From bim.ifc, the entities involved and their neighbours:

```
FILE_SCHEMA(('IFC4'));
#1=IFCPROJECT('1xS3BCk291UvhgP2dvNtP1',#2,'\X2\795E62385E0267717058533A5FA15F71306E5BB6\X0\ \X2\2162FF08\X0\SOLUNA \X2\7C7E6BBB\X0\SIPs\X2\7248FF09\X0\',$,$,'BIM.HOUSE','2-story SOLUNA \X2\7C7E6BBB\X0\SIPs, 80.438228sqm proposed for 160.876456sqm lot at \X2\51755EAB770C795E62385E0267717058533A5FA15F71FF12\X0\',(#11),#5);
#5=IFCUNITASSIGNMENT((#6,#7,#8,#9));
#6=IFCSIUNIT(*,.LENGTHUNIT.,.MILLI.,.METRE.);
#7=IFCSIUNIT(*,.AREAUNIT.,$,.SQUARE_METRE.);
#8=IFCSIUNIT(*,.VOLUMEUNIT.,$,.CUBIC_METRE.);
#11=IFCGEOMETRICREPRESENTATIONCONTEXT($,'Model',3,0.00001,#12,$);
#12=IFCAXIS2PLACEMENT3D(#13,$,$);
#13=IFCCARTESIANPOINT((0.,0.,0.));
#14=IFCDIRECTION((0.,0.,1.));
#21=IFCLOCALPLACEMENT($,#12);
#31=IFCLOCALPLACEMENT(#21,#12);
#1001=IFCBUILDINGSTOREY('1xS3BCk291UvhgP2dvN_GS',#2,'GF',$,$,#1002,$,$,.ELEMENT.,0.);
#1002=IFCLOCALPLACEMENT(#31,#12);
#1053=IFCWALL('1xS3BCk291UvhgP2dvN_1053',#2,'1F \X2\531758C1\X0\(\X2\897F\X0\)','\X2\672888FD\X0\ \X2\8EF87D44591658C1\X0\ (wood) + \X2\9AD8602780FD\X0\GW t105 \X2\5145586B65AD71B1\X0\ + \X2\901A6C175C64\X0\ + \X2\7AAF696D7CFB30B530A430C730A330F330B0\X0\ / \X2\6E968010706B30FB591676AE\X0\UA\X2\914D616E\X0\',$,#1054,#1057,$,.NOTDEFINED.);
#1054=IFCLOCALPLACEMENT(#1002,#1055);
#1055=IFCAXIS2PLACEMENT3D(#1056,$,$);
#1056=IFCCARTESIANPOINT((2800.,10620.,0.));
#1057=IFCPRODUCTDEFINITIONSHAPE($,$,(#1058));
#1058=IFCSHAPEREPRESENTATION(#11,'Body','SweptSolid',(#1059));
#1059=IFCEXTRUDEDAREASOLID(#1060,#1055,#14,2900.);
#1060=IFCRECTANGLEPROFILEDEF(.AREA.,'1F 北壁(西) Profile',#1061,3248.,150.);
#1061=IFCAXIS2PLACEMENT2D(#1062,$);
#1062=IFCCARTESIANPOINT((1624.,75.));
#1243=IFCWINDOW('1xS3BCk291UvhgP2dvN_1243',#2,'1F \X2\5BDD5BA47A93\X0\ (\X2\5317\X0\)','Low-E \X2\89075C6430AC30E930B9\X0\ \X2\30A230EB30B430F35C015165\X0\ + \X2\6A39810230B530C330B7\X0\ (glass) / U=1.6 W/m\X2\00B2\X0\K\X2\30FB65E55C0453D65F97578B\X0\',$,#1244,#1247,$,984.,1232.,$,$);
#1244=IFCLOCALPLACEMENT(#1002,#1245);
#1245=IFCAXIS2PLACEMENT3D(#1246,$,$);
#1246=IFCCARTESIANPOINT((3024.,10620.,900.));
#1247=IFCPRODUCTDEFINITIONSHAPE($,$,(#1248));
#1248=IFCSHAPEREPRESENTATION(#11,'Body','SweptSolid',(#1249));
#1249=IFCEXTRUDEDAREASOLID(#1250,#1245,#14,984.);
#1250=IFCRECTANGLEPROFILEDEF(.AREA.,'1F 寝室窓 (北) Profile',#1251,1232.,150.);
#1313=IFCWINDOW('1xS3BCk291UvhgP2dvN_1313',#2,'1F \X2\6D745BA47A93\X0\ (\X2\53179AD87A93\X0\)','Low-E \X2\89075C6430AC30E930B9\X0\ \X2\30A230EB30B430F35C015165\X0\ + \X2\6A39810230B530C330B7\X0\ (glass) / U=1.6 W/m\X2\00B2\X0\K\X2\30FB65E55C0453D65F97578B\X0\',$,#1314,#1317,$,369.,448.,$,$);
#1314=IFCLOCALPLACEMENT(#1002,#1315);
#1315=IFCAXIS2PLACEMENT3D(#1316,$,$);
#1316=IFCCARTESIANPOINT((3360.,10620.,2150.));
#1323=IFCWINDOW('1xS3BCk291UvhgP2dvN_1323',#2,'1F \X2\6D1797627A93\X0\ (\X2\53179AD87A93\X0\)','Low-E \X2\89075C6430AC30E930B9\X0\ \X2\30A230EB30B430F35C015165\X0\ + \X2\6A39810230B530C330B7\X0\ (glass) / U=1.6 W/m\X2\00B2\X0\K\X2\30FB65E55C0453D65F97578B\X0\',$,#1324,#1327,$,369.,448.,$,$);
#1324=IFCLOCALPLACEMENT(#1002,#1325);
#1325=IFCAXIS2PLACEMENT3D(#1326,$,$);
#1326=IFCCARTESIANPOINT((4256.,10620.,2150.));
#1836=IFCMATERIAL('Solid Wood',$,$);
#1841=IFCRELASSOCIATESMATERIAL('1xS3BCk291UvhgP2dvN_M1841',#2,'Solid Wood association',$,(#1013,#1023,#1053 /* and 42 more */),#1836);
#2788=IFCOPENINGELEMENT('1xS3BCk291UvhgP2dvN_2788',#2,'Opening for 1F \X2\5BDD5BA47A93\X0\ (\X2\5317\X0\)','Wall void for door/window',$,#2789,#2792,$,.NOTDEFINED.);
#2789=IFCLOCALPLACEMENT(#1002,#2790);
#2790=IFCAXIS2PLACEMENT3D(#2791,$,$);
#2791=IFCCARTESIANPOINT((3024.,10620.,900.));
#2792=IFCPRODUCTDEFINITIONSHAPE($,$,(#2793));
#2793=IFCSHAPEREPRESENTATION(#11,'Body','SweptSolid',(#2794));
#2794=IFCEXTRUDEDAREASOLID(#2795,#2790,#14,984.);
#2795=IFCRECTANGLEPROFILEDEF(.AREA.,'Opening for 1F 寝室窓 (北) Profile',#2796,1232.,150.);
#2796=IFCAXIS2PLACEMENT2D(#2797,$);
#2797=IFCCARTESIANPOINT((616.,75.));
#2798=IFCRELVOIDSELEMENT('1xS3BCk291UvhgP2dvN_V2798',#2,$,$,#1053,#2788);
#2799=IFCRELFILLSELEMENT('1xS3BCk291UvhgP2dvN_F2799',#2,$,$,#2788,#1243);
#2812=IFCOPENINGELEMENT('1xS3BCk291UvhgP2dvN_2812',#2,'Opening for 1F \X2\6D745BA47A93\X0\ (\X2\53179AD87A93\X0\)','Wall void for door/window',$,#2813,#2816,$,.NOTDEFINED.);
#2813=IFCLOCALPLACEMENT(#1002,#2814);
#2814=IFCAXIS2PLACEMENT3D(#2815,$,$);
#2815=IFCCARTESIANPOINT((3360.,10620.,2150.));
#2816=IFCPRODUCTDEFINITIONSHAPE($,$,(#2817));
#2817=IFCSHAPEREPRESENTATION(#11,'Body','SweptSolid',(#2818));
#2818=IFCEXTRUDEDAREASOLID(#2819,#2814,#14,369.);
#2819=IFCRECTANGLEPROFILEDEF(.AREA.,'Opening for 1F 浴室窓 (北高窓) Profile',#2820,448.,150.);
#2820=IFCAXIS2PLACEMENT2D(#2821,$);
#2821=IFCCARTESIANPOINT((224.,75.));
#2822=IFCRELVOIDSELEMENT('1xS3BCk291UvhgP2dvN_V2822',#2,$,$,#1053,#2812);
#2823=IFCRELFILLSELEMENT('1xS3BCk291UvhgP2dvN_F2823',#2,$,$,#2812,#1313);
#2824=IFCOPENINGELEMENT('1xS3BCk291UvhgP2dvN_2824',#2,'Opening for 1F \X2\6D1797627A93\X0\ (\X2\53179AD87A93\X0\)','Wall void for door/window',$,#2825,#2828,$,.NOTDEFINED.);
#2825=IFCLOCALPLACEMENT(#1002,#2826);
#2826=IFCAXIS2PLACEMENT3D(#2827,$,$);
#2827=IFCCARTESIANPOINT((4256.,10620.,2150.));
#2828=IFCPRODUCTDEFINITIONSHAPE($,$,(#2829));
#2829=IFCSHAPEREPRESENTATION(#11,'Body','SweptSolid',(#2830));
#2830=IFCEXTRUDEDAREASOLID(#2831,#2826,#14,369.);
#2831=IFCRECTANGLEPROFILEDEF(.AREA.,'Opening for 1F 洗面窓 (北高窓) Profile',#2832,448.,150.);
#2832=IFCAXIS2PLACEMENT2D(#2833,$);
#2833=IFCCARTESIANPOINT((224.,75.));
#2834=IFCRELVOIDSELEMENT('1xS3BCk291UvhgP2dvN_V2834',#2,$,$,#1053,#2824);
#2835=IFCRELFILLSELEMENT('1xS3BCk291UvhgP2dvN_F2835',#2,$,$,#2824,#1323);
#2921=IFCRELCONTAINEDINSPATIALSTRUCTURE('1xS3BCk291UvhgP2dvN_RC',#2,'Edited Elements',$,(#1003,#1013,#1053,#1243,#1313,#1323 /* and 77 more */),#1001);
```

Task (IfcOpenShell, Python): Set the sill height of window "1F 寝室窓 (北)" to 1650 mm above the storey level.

```python
import numpy as np
import ifcopenshell
import ifcopenshell.api.geometry
import ifcopenshell.geom
import ifcopenshell.util.element
import ifcopenshell.util.placement
import ifcopenshell.util.shape
import ifcopenshell.util.unit

model = ifcopenshell.open("bim.ifc")
unit_scale = ifcopenshell.util.unit.calculate_unit_scale(model)

window = model.by_guid("1xS3BCk291UvhgP2dvN_1243")
opening = window.FillsVoids[0].RelatingOpeningElement
storey = ifcopenshell.util.element.get_container(window, ifc_class="IfcBuildingStorey")
level = ifcopenshell.util.placement.get_local_placement(storey.ObjectPlacement)[2, 3]

# The opening's origin need not be at the sill, so measure its lowest point.
shape = ifcopenshell.geom.create_shape(ifcopenshell.geom.settings(), opening)
bottom = ifcopenshell.util.shape.get_shape_bottom_elevation(shape, shape.geometry) / unit_scale
dz = level + 1.65 / unit_scale - bottom

shift = np.array([0.0, 0.0, dz])
# The window is not placed relative to its opening, so move both.
for product in (opening, window):
    matrix = ifcopenshell.util.placement.get_local_placement(product.ObjectPlacement)
    matrix[:3, 3] += shift
    ifcopenshell.api.geometry.edit_object_placement(model, product=product, matrix=matrix, is_si=False)

print(f"moved by {dz * unit_scale:+.3f} m")

model.write("bim_v2.ifc")
```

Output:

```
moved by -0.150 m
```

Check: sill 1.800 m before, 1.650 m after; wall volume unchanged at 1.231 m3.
